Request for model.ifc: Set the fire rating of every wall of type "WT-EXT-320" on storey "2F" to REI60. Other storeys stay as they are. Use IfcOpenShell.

First a look at what the model holds.

```python
import ifcopenshell
import ifcopenshell.util.element

model = ifcopenshell.open("model.ifc")
print(model.schema)
storey = next(s for s in model.by_type("IfcBuildingStorey") if s.Name == "2F")
walls = [e for e in ifcopenshell.util.element.get_decomposition(storey) if e.is_a("IfcWall")]
seen = {}
for e in walls:
    element_type = ifcopenshell.util.element.get_type(e)
    key = (element_type.Name if element_type != e and element_type else None, ifcopenshell.util.element.get_pset(e, "Pset_WallCommon", "FireRating"))
    seen[key] = seen.get(key, 0) + 1
for (name, value), count in sorted(seen.items(), key=str):
    print(count, "x", name, "|", value)
```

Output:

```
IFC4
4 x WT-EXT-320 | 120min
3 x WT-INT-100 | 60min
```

```python
import ifcopenshell
import ifcopenshell.api.pset
import ifcopenshell.util.element

model = ifcopenshell.open("model.ifc")

storey = next(s for s in model.by_type("IfcBuildingStorey") if s.Name == "2F")
walls = [e for e in ifcopenshell.util.element.get_decomposition(storey) if e.is_a("IfcWall")]

count = 0
for e in walls:
    element_type = ifcopenshell.util.element.get_type(e)
    if element_type in (None, e) or element_type.Name != "WT-EXT-320":
        continue
    # add_pset returns the element's existing set when there is one.
    pset = ifcopenshell.api.pset.add_pset(model, product=e, name="Pset_WallCommon")
    ifcopenshell.api.pset.edit_pset(model, pset=pset, properties={"FireRating": "REI60"})
    count += 1

print(count, "walls updated")

model.write("model_v2.ifc")
```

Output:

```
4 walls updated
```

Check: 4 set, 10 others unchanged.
